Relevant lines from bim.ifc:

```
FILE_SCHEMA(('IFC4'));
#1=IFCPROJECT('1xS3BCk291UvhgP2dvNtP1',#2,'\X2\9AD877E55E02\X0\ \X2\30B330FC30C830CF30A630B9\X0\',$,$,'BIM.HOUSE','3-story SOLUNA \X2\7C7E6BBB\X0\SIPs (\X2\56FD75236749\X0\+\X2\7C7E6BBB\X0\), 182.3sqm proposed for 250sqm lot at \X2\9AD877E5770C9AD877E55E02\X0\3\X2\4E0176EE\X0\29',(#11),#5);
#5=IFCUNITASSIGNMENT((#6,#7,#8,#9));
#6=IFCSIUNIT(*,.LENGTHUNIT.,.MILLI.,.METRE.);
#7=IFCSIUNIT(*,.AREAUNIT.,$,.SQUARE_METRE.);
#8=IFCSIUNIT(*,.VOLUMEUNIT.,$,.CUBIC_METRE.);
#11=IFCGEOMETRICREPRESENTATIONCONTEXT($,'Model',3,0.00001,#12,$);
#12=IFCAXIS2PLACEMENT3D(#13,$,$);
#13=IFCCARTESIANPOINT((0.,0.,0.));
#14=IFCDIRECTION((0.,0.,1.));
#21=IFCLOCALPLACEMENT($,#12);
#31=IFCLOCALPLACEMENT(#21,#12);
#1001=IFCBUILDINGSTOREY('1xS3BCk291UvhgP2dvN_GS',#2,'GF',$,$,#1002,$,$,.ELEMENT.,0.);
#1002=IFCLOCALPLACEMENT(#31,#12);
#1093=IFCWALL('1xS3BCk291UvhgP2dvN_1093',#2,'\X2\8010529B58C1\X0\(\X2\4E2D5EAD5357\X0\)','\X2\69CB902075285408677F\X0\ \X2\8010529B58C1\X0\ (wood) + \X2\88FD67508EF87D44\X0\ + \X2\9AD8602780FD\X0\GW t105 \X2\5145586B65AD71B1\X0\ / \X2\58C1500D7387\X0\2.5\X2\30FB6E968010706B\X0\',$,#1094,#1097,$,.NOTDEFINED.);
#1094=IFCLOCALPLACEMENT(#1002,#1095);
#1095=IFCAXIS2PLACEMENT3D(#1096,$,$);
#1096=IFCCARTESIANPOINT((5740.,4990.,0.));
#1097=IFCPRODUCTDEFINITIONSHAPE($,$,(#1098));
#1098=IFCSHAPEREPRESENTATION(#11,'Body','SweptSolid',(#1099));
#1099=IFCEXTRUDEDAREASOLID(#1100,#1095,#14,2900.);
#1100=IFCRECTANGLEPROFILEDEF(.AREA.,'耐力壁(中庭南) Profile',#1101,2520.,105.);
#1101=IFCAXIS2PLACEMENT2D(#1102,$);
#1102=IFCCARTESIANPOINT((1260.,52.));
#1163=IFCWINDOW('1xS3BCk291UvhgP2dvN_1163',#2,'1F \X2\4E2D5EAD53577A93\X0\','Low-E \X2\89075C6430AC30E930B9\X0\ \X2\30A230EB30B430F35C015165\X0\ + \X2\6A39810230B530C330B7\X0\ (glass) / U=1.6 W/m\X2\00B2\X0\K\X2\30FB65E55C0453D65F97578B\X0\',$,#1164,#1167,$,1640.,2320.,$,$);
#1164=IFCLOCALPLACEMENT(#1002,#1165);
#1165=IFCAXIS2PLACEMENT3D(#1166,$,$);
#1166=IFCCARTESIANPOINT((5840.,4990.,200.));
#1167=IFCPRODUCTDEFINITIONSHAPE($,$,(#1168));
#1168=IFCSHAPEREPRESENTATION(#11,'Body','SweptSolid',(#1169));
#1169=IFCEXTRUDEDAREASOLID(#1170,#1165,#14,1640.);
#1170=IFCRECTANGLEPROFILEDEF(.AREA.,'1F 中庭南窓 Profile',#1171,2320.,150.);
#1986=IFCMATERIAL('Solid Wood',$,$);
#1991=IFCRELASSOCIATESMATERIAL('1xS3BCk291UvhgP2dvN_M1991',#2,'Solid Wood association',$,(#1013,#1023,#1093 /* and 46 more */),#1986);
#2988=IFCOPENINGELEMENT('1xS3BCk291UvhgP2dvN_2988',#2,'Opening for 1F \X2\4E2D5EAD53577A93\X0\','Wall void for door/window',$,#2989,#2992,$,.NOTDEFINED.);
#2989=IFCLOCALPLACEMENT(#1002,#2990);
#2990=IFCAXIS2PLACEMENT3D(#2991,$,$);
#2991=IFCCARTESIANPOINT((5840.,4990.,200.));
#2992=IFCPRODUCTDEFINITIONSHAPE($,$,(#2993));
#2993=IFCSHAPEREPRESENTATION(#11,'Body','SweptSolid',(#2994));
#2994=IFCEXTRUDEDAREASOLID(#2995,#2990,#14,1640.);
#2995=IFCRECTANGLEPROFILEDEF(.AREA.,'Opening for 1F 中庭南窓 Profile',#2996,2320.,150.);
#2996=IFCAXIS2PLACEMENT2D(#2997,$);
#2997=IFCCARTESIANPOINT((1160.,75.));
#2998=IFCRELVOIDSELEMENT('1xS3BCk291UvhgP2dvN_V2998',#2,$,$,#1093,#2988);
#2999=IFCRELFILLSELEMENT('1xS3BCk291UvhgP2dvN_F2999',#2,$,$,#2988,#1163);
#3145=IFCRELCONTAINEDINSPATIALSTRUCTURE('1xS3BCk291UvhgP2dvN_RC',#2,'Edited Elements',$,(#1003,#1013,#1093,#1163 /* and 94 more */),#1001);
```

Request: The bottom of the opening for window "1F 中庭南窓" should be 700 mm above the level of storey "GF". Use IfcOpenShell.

```python
import numpy as np
import ifcopenshell
import ifcopenshell.api.geometry
import ifcopenshell.geom
import ifcopenshell.util.element
import ifcopenshell.util.placement
import ifcopenshell.util.shape
import ifcopenshell.util.unit

model = ifcopenshell.open("bim.ifc")
unit_scale = ifcopenshell.util.unit.calculate_unit_scale(model)

window = model.by_guid("1xS3BCk291UvhgP2dvN_1163")
opening = window.FillsVoids[0].RelatingOpeningElement
storey = ifcopenshell.util.element.get_container(window, ifc_class="IfcBuildingStorey")
level = ifcopenshell.util.placement.get_local_placement(storey.ObjectPlacement)[2, 3]

# The opening's origin need not be at the sill, so measure its lowest point.
shape = ifcopenshell.geom.create_shape(ifcopenshell.geom.settings(), opening)
bottom = ifcopenshell.util.shape.get_shape_bottom_elevation(shape, shape.geometry) / unit_scale
dz = level + 700.0 - bottom

shift = np.array([0.0, 0.0, dz])
# The window is not placed relative to its opening, so move both.
for product in (opening, window):
    matrix = ifcopenshell.util.placement.get_local_placement(product.ObjectPlacement)
    matrix[:3, 3] += shift
    ifcopenshell.api.geometry.edit_object_placement(model, product=product, matrix=matrix, is_si=False)

print(f"moved by {dz * unit_scale:+.3f} m")

model.write("bim_v2.ifc")
```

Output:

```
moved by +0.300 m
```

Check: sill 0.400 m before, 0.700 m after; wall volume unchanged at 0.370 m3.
